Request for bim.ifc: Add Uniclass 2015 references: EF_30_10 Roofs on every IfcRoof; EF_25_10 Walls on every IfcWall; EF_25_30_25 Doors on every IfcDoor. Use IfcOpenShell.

First a look at what the model holds.

```python
import ifcopenshell

model = ifcopenshell.open("bim.ifc")
print(model.schema)
print("classifications:", [c.Name for c in model.by_type("IfcClassification")])
for ifc_class in ("IfcDoor", "IfcRoof", "IfcStair", "IfcWall", "IfcWindow"):
    print(ifc_class, len(model.by_type(ifc_class)))
```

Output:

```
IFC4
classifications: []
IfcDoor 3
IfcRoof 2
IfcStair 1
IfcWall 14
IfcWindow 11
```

```python
import ifcopenshell
import ifcopenshell.api.classification

model = ifcopenshell.open("bim.ifc")

system = ifcopenshell.api.classification.add_classification(model, classification="Uniclass 2015")

codes = {
    "IfcRoof": ("EF_30_10", "Roofs"),
    "IfcWall": ("EF_25_10", "Walls"),
    "IfcDoor": ("EF_25_30_25", "Doors"),
}
for ifc_class, (code, name) in codes.items():
    products = model.by_type(ifc_class)
    ifcopenshell.api.classification.add_reference(
        model, products=products, classification=system, identification=code, name=name
    )
    print(code, len(products))

model.write("bim_edited.ifc")
```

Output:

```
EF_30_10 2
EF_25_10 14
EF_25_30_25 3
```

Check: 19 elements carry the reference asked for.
